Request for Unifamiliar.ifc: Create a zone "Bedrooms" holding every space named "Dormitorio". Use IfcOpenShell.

First a look at what the model holds.

```python
import ifcopenshell

model = ifcopenshell.open("Unifamiliar.ifc")
print(model.schema)
seen = {}
for space in model.by_type("IfcSpace"):
    seen[space.LongName] = seen.get(space.LongName, 0) + 1
for name, count in sorted(seen.items(), key=str):
    print(count, "x", name)
print("zones:", [z.Name for z in model.by_type("IfcZone")][:20])
```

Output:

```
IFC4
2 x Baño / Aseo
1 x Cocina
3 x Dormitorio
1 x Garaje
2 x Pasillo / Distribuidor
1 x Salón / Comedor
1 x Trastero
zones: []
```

```python
import ifcopenshell
import ifcopenshell.api.group
import ifcopenshell.api.root

model = ifcopenshell.open("Unifamiliar.ifc")

names = {"Dormitorio"}
spaces = [s for s in model.by_type("IfcSpace") if s.LongName in names]

zone = ifcopenshell.api.root.create_entity(model, ifc_class="IfcZone", name="Bedrooms")
ifcopenshell.api.group.assign_group(model, products=spaces, group=zone)
print(len(spaces), "spaces in", zone.Name)

model.write("Unifamiliar_edited.ifc")
```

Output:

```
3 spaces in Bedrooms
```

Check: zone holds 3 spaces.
